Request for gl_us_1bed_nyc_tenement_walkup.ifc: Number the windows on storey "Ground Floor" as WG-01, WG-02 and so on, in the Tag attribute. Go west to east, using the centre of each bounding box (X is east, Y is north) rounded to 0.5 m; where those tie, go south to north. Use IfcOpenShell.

First a look at what the model holds.

```python
import ifcopenshell
import ifcopenshell.util.element
import ifcopenshell.util.placement

model = ifcopenshell.open("gl_us_1bed_nyc_tenement_walkup.ifc")
print(model.schema)
storey = next(s for s in model.by_type("IfcBuildingStorey") if s.Name == "Ground Floor")
windows = [e for e in ifcopenshell.util.element.get_decomposition(storey) if e.is_a("IfcWindow")]
for e in sorted(windows, key=lambda e: e.id()):
    origin = ifcopenshell.util.placement.get_local_placement(e.ObjectPlacement)[:3, 3]
    print(e.id(), e.Tag, e.Name, origin.round(2) + 0.0, sep=" | ")
```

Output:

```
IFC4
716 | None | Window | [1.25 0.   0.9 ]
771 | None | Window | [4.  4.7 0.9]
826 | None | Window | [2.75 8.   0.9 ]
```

```python
import ifcopenshell
import ifcopenshell.geom
import ifcopenshell.util.element
import ifcopenshell.util.shape

model = ifcopenshell.open("gl_us_1bed_nyc_tenement_walkup.ifc")
settings = ifcopenshell.geom.settings()
settings.set("use-world-coords", True)


def centre(element):
    shape = ifcopenshell.geom.create_shape(settings, element)
    return ifcopenshell.util.shape.get_bbox_centroid(shape.geometry)


storey = next(s for s in model.by_type("IfcBuildingStorey") if s.Name == "Ground Floor")
windows = [e for e in ifcopenshell.util.element.get_decomposition(storey) if e.is_a("IfcWindow")]

# Insertion points can sit at a corner or the storey origin, so sort by the geometry (in metres).
centres = {e: centre(e) for e in windows}
windows.sort(key=lambda e: (round(centres[e][0] / 0.5), centres[e][1]))

for i, e in enumerate(windows, start=1):
    number = f"WG-{i:02d}"
    e.Tag = number
    print(e.id(), number)

model.write("gl_us_1bed_nyc_tenement_walkup-out.ifc")
```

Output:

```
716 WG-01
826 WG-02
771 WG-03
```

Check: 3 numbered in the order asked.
